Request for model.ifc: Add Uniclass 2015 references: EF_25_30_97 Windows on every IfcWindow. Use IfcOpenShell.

First a look at what the model holds.

```python
import ifcopenshell

model = ifcopenshell.open("model.ifc")
print(model.schema)
print("classifications:", [c.Name for c in model.by_type("IfcClassification")])
for ifc_class in ("IfcDoor", "IfcRoof", "IfcStair", "IfcWall", "IfcWindow"):
    print(ifc_class, len(model.by_type(ifc_class)))
```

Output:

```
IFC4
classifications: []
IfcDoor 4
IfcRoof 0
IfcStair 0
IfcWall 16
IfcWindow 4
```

```python
import ifcopenshell
import ifcopenshell.api.classification

model = ifcopenshell.open("model.ifc")

system = ifcopenshell.api.classification.add_classification(model, classification="Uniclass 2015")

codes = {
    "IfcWindow": ("EF_25_30_97", "Windows"),
}
for ifc_class, (code, name) in codes.items():
    products = model.by_type(ifc_class)
    ifcopenshell.api.classification.add_reference(
        model, products=products, classification=system, identification=code, name=name
    )
    print(code, len(products))

model.write("model_rev.ifc")
```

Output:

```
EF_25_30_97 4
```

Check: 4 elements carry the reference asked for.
